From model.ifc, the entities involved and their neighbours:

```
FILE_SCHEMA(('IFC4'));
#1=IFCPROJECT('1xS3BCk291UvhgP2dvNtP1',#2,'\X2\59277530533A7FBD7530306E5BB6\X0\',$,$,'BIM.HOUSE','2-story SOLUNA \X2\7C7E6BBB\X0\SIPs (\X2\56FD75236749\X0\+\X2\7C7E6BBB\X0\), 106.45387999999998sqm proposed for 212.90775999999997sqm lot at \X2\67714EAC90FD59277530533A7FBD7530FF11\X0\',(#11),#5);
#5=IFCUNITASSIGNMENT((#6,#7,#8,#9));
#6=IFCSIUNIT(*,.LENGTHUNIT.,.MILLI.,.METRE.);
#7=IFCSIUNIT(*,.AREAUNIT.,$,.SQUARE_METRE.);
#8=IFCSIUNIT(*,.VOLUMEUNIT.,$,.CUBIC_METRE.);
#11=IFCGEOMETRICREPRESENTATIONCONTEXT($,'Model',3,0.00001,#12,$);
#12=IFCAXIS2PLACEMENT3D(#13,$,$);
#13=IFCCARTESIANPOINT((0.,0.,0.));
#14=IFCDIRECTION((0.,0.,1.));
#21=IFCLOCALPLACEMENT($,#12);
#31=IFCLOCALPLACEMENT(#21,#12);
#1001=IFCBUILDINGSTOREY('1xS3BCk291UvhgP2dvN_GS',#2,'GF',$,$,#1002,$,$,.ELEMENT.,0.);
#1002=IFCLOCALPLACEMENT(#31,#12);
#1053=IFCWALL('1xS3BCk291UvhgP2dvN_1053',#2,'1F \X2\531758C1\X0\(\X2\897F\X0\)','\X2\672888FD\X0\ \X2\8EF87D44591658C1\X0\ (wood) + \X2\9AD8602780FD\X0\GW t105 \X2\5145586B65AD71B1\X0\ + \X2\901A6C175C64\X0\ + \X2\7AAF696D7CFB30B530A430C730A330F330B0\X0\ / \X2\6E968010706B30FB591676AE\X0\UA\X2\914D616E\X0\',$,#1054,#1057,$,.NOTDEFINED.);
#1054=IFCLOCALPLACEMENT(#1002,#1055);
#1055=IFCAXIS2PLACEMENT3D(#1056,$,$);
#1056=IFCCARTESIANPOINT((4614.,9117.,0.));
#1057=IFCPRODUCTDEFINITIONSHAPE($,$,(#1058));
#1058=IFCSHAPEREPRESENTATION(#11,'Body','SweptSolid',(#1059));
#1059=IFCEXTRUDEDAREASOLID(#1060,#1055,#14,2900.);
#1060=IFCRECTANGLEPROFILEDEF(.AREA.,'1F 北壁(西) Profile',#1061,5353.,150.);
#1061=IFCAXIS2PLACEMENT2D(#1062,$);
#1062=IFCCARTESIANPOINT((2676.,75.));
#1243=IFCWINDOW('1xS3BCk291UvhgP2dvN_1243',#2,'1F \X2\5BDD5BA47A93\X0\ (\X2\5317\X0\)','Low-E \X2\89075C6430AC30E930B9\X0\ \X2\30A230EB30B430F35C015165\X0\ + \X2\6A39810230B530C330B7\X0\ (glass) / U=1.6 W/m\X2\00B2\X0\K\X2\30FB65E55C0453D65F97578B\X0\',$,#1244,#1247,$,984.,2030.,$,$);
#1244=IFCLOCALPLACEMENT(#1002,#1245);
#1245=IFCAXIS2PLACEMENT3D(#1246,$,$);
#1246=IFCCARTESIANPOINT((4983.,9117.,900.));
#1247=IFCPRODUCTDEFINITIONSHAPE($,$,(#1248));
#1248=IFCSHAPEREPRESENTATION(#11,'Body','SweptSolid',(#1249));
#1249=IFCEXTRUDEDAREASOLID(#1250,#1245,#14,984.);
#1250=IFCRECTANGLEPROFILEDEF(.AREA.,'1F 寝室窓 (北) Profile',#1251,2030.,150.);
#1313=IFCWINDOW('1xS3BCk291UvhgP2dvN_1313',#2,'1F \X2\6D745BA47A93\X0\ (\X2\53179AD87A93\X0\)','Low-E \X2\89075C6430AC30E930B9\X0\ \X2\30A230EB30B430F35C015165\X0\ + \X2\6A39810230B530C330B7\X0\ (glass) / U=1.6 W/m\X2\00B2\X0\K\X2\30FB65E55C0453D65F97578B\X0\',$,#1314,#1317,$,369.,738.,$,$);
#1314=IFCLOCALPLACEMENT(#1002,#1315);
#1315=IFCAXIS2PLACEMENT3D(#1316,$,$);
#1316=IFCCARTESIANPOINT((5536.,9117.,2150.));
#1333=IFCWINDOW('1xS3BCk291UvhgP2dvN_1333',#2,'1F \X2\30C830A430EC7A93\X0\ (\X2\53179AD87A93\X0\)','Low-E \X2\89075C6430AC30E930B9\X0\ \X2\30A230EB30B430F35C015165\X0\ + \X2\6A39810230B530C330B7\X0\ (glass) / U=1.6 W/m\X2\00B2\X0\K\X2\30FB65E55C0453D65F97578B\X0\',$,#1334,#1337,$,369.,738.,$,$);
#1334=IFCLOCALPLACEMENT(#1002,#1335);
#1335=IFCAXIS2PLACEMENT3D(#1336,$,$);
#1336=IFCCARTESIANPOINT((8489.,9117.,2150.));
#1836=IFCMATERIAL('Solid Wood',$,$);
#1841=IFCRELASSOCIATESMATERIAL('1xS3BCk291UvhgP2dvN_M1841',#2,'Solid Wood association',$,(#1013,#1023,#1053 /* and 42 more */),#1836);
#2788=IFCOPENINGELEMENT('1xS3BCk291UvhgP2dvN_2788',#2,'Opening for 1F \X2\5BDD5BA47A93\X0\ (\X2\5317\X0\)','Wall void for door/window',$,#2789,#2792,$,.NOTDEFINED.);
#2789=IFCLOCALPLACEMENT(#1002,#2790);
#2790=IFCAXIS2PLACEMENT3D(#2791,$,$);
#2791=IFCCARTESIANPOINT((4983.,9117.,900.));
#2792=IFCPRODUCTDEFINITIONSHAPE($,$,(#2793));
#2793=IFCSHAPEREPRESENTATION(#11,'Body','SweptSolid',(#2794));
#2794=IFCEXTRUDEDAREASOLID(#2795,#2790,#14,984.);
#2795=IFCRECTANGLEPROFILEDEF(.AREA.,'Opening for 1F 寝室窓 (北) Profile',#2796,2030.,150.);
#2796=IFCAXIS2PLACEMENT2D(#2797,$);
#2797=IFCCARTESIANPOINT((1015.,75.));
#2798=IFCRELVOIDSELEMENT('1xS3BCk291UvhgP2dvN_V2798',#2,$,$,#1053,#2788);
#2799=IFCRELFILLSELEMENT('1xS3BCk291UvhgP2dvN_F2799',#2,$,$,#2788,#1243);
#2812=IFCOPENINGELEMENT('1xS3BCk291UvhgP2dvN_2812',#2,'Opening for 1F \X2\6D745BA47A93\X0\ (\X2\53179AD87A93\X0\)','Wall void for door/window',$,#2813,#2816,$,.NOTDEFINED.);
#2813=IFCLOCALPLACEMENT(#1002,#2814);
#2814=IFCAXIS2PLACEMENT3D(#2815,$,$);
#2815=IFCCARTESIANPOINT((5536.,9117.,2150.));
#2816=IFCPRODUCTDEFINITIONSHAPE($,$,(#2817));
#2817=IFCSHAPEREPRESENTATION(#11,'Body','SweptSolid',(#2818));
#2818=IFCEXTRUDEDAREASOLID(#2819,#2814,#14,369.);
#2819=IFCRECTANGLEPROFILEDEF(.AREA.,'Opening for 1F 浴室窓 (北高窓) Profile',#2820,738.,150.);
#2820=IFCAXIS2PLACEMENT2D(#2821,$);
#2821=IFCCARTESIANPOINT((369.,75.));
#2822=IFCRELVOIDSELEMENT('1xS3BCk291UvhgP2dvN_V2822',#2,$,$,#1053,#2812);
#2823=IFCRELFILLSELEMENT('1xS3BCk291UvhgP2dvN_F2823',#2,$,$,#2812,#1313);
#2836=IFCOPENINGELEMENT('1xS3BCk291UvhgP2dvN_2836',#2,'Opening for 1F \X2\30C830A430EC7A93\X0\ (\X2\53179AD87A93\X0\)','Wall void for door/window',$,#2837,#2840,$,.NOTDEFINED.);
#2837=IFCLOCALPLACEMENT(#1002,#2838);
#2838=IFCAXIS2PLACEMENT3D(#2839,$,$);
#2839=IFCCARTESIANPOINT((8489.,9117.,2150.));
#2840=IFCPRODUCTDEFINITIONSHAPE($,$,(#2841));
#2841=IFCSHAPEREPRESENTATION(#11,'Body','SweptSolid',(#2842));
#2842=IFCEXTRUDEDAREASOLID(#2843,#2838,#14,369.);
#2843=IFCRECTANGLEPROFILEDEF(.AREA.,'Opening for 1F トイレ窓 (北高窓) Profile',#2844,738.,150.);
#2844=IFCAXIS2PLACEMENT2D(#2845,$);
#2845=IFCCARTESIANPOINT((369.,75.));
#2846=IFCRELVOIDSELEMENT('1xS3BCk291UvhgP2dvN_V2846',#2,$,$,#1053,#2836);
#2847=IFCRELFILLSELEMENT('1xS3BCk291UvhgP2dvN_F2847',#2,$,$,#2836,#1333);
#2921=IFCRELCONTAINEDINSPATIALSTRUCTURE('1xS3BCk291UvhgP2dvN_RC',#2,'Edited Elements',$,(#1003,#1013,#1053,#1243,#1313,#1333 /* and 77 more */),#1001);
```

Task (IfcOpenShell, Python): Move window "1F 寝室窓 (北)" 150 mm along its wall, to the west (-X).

```python
import ifcopenshell
import ifcopenshell.api.geometry
import ifcopenshell.util.placement
import ifcopenshell.util.unit

model = ifcopenshell.open("model.ifc")
unit_scale = ifcopenshell.util.unit.calculate_unit_scale(model)

window = model.by_guid("1xS3BCk291UvhgP2dvN_1243")
opening = window.FillsVoids[0].RelatingOpeningElement
wall = opening.VoidsElements[0].RelatingBuildingElement

wall_matrix = ifcopenshell.util.placement.get_local_placement(wall.ObjectPlacement)
shift = wall_matrix[:3, 0] * -0.15 / unit_scale
before = ifcopenshell.util.placement.get_local_placement(window.ObjectPlacement)[:3, 3].copy()

# The window is not placed relative to its opening, so move both.
for product in (opening, window):
    matrix = ifcopenshell.util.placement.get_local_placement(product.ObjectPlacement)
    matrix[:3, 3] += shift
    ifcopenshell.api.geometry.edit_object_placement(model, product=product, matrix=matrix, is_si=False)

after = ifcopenshell.util.placement.get_local_placement(window.ObjectPlacement)[:3, 3]
print("window moved by", (after - before).round(3) + 0.0)

model.write("model_rev.ifc")
```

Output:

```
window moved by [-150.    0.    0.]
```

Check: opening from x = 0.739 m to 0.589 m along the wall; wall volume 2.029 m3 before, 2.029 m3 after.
